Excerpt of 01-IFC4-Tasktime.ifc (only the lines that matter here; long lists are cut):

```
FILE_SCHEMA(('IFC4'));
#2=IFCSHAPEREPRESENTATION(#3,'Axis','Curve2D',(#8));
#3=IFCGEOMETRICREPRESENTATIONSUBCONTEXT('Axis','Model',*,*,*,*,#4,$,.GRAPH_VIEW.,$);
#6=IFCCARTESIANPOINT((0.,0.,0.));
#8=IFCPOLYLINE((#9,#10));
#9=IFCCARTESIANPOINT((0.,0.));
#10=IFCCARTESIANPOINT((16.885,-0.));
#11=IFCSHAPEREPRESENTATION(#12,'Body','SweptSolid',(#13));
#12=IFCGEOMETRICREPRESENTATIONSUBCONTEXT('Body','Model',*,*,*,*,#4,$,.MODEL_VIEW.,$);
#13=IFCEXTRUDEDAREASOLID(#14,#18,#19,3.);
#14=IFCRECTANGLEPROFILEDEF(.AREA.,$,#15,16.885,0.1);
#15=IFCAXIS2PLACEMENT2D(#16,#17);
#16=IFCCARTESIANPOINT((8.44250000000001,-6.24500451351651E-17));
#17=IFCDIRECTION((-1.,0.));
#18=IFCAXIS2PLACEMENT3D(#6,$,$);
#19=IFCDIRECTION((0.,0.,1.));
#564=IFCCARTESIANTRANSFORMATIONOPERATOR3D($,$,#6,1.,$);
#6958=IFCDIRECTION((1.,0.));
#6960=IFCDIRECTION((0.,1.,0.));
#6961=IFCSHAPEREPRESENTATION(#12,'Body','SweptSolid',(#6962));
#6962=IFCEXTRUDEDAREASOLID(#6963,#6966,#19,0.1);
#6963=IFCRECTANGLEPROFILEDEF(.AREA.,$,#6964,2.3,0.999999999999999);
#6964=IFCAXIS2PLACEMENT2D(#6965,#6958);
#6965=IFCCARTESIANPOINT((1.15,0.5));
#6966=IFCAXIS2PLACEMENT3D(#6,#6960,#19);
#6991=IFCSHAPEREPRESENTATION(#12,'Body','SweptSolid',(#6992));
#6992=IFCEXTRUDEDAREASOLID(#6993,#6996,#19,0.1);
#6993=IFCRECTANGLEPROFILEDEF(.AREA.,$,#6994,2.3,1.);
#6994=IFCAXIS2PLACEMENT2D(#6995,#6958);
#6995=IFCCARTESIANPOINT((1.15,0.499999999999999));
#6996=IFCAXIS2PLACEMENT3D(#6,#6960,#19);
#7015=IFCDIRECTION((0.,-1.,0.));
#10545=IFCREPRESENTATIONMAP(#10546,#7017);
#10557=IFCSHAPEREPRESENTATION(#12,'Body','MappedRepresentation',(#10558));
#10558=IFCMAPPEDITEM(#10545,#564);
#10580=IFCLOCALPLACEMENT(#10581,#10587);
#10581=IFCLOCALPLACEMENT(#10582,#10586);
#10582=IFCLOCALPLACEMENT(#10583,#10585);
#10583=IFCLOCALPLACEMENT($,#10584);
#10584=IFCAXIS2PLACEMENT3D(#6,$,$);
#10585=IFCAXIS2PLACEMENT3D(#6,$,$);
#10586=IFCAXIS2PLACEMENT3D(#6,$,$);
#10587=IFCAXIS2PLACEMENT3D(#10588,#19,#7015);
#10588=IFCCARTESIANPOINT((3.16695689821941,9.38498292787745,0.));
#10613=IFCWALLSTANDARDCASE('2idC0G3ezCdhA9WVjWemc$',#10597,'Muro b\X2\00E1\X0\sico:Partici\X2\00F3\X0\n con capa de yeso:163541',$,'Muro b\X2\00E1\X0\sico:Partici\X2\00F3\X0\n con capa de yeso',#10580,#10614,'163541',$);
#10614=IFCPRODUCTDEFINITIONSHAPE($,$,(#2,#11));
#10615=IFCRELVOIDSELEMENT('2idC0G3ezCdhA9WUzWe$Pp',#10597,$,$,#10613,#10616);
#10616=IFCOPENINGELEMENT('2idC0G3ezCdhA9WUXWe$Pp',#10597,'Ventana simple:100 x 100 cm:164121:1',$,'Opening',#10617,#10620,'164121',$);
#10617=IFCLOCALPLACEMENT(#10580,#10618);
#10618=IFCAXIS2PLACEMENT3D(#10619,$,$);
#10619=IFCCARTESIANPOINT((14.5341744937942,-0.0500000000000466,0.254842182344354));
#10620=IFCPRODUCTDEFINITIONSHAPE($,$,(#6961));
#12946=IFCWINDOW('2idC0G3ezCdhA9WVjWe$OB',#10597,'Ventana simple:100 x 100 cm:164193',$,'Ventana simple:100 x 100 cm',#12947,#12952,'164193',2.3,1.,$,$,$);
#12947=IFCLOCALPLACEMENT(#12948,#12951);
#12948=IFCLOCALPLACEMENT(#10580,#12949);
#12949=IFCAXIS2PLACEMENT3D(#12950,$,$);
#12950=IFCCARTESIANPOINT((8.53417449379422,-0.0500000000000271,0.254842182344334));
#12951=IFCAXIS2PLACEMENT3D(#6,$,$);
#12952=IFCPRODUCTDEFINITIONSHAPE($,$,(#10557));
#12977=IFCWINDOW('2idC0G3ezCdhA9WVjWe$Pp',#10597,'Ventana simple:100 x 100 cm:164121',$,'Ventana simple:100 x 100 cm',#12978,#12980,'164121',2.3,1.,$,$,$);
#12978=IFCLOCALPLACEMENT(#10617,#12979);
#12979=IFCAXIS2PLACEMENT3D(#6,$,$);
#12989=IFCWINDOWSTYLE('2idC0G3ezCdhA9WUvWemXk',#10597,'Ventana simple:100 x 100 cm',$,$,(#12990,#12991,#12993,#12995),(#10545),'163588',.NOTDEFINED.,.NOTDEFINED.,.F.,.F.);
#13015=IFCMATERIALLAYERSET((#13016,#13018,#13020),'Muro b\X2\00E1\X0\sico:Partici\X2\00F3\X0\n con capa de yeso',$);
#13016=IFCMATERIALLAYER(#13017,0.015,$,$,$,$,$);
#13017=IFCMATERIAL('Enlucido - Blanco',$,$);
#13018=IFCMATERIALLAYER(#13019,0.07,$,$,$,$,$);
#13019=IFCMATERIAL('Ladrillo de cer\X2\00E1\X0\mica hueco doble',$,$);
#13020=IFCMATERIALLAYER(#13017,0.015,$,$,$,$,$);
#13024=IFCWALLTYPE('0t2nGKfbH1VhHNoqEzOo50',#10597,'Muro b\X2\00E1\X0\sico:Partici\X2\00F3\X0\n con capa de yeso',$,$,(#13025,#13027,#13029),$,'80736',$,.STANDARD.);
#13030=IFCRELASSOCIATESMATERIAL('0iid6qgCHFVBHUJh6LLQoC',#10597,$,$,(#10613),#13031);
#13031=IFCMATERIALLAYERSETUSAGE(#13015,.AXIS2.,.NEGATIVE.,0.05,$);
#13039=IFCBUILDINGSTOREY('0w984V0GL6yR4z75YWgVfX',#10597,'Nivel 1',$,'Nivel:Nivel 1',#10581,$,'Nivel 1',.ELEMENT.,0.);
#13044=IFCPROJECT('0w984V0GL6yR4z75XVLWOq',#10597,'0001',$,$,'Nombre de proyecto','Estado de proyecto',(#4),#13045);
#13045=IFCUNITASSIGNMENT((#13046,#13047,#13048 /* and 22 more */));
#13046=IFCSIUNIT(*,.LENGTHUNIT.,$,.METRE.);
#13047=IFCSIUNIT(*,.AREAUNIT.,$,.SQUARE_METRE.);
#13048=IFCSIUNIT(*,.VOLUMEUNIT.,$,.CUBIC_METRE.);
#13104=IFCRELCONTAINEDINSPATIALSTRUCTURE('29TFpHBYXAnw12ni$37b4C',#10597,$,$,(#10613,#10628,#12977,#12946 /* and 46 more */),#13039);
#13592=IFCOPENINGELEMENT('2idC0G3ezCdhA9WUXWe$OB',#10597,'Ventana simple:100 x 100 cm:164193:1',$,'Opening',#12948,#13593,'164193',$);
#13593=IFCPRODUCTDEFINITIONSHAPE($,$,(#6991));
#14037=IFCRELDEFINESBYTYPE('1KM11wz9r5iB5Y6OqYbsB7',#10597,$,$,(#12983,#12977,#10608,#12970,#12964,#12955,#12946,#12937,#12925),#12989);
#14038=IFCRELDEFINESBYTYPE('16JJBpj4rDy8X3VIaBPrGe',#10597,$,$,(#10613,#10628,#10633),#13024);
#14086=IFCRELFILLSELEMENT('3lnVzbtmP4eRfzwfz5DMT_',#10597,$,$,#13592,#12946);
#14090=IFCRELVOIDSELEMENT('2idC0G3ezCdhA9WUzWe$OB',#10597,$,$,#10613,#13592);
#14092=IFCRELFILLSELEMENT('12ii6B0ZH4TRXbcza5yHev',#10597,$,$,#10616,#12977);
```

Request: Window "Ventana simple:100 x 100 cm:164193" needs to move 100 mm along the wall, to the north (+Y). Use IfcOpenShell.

```python
import ifcopenshell
import ifcopenshell.api.geometry
import ifcopenshell.util.placement
import ifcopenshell.util.unit

model = ifcopenshell.open("01-IFC4-Tasktime.ifc")
unit_scale = ifcopenshell.util.unit.calculate_unit_scale(model)

window = model.by_guid("2idC0G3ezCdhA9WVjWe$OB")
opening = window.FillsVoids[0].RelatingOpeningElement
wall = opening.VoidsElements[0].RelatingBuildingElement

wall_matrix = ifcopenshell.util.placement.get_local_placement(wall.ObjectPlacement)
shift = wall_matrix[:3, 0] * -0.1 / unit_scale
before = ifcopenshell.util.placement.get_local_placement(window.ObjectPlacement)[:3, 3].copy()

# The window is placed relative to its opening, so it follows when the opening moves.
matrix = ifcopenshell.util.placement.get_local_placement(opening.ObjectPlacement)
matrix[:3, 3] += shift
ifcopenshell.api.geometry.edit_object_placement(
    model, product=opening, matrix=matrix, is_si=False, should_transform_children=True
)

after = ifcopenshell.util.placement.get_local_placement(window.ObjectPlacement)[:3, 3]
print("window moved by", (after - before).round(3) + 0.0)

model.write("01-IFC4-Tasktime-out.ifc")
```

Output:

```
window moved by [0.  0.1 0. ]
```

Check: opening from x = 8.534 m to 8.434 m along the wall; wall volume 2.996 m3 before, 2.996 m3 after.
